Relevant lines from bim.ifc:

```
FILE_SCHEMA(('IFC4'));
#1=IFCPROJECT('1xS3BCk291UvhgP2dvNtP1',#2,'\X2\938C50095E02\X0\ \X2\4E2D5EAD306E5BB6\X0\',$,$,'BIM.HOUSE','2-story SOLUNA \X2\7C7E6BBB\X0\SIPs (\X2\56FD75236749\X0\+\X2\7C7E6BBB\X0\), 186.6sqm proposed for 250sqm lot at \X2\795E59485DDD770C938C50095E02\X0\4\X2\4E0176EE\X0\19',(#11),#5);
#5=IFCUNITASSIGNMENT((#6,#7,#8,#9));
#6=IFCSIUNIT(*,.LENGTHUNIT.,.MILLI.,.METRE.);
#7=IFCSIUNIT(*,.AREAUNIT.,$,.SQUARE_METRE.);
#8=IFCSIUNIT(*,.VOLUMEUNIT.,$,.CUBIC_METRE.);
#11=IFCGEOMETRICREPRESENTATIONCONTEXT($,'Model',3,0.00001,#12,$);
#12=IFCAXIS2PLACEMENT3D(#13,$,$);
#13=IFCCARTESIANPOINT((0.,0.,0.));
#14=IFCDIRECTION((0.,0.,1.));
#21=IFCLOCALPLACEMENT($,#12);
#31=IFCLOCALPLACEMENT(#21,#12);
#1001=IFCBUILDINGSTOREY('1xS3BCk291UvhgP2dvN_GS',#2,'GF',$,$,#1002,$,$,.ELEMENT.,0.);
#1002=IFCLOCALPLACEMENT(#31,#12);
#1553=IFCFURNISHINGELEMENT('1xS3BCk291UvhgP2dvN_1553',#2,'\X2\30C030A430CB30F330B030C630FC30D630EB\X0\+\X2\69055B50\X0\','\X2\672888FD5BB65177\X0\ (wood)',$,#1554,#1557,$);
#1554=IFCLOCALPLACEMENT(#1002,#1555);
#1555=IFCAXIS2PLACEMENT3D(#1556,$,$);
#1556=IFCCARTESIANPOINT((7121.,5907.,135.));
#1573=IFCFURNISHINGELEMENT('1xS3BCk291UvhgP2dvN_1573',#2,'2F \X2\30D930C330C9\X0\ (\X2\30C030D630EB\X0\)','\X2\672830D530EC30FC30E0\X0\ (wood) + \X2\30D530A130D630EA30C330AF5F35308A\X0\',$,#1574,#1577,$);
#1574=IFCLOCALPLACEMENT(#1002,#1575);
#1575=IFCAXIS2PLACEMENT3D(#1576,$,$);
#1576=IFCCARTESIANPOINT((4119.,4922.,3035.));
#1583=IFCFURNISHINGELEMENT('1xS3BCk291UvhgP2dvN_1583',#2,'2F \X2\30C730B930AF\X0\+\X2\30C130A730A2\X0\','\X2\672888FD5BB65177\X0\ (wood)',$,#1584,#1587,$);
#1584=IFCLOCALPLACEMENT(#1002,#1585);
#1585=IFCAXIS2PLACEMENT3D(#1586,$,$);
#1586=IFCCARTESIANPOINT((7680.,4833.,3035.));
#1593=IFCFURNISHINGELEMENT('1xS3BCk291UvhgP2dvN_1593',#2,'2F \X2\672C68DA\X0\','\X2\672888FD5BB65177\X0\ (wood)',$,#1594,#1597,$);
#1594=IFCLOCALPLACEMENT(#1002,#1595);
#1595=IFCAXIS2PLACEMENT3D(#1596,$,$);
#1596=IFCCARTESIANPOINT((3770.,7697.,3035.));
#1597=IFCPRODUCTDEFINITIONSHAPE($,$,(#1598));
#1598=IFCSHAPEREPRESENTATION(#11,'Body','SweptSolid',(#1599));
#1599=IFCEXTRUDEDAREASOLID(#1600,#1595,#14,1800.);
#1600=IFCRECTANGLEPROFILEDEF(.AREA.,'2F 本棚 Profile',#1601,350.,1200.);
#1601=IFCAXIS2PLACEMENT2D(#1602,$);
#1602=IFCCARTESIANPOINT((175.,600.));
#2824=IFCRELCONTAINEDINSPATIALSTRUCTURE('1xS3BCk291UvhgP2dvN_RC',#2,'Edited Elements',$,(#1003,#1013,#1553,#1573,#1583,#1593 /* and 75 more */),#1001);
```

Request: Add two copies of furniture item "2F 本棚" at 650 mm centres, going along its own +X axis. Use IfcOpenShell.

```python
import ifcopenshell
import ifcopenshell.api.geometry
import ifcopenshell.api.root
import ifcopenshell.util.element
import ifcopenshell.util.placement

model = ifcopenshell.open("bim.ifc")


def reuse_history(source, copy):
    """copy_class also copies each property set's owner history, people and application; keep the originals."""
    for rel in copy.IsDefinedBy:
        if rel.is_a("IfcRelDefinesByProperties") and (history := rel.RelatingPropertyDefinition.OwnerHistory):
            rel.RelatingPropertyDefinition.OwnerHistory = source.OwnerHistory
            ifcopenshell.util.element.remove_deep2(model, history)


source = model.by_guid("1xS3BCk291UvhgP2dvN_1593")
base = ifcopenshell.util.placement.get_local_placement(source.ObjectPlacement)
step = base[:3, 0] * 650.0

for i in range(1, 3):
    copy = ifcopenshell.api.root.copy_class(model, product=source)
    copy.Representation = ifcopenshell.util.element.copy_deep(
        model, source.Representation, exclude=["IfcGeometricRepresentationContext", "IfcRepresentationMap"]
    )
    reuse_history(source, copy)
    matrix = base.copy()
    matrix[:3, 3] += i * step
    print("added at", matrix[:3, 3].round(3) + 0.0)
    ifcopenshell.api.geometry.edit_object_placement(model, product=copy, matrix=matrix, is_si=False)

model.write("bim_updated.ifc")
```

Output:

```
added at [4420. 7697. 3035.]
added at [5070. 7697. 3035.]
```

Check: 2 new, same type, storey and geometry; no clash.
